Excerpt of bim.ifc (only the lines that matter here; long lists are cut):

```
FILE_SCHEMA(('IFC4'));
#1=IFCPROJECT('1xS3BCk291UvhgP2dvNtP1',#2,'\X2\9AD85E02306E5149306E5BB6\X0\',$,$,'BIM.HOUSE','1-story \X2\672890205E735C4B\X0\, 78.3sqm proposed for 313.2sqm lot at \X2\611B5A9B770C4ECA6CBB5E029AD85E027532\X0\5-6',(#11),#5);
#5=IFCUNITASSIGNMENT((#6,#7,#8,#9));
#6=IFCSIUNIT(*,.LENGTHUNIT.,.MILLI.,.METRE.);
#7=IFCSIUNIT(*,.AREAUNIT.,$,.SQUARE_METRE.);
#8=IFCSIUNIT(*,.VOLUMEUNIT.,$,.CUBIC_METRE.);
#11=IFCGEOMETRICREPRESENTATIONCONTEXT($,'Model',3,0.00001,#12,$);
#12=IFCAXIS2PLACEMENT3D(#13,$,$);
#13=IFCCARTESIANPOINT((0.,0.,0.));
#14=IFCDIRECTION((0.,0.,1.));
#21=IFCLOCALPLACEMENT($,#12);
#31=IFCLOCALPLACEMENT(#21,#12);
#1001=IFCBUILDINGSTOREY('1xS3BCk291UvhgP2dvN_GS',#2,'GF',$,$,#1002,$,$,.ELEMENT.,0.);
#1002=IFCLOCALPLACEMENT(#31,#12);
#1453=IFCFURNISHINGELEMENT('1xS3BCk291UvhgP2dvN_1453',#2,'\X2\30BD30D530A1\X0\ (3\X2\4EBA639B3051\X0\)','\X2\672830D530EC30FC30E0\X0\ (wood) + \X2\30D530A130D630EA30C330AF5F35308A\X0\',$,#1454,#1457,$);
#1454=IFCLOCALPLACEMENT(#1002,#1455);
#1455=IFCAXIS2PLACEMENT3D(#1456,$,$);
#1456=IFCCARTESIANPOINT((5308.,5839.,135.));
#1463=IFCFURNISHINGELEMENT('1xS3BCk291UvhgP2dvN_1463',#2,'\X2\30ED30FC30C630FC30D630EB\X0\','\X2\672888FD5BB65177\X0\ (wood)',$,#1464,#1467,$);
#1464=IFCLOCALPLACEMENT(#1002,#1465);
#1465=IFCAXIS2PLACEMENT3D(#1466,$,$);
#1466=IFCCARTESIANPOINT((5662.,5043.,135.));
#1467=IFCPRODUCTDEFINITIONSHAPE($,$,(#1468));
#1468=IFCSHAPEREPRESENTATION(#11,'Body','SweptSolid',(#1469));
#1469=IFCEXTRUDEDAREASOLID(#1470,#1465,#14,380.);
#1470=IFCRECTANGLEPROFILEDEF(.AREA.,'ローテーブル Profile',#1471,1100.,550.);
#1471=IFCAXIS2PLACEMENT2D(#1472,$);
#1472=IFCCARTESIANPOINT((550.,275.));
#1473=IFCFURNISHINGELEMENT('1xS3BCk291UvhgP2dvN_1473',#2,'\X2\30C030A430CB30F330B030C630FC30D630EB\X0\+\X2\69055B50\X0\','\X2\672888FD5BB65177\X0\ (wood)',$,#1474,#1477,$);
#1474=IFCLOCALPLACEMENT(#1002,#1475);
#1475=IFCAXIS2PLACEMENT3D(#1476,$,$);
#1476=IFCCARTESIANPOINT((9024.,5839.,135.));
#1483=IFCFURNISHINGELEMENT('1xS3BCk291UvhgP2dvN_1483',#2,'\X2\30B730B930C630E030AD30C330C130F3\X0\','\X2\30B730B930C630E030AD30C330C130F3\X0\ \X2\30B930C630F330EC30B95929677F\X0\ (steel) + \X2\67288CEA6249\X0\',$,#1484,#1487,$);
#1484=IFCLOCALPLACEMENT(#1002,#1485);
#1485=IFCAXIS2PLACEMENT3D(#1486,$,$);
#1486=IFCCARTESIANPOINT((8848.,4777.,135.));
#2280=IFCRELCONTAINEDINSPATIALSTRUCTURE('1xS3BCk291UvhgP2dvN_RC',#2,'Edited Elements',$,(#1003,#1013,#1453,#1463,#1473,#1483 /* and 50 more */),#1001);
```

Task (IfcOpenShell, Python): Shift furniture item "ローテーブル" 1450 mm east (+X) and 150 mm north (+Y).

```python
import ifcopenshell
import ifcopenshell.api.geometry
import ifcopenshell.util.placement
import ifcopenshell.util.unit

model = ifcopenshell.open("bim.ifc")
unit_scale = ifcopenshell.util.unit.calculate_unit_scale(model)

item = model.by_guid("1xS3BCk291UvhgP2dvN_1463")
matrix = ifcopenshell.util.placement.get_local_placement(item.ObjectPlacement)
matrix[0, 3] += 1.45 / unit_scale
matrix[1, 3] += 0.15 / unit_scale
ifcopenshell.api.geometry.edit_object_placement(model, product=item, matrix=matrix, is_si=False)

print(ifcopenshell.util.placement.get_local_placement(item.ObjectPlacement).round(3) + 0.0)

model.write("bim_rev.ifc")
```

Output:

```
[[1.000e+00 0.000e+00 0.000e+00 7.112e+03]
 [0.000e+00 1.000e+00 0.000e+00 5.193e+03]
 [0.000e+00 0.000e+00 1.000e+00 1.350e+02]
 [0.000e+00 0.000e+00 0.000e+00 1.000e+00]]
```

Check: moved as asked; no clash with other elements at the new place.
